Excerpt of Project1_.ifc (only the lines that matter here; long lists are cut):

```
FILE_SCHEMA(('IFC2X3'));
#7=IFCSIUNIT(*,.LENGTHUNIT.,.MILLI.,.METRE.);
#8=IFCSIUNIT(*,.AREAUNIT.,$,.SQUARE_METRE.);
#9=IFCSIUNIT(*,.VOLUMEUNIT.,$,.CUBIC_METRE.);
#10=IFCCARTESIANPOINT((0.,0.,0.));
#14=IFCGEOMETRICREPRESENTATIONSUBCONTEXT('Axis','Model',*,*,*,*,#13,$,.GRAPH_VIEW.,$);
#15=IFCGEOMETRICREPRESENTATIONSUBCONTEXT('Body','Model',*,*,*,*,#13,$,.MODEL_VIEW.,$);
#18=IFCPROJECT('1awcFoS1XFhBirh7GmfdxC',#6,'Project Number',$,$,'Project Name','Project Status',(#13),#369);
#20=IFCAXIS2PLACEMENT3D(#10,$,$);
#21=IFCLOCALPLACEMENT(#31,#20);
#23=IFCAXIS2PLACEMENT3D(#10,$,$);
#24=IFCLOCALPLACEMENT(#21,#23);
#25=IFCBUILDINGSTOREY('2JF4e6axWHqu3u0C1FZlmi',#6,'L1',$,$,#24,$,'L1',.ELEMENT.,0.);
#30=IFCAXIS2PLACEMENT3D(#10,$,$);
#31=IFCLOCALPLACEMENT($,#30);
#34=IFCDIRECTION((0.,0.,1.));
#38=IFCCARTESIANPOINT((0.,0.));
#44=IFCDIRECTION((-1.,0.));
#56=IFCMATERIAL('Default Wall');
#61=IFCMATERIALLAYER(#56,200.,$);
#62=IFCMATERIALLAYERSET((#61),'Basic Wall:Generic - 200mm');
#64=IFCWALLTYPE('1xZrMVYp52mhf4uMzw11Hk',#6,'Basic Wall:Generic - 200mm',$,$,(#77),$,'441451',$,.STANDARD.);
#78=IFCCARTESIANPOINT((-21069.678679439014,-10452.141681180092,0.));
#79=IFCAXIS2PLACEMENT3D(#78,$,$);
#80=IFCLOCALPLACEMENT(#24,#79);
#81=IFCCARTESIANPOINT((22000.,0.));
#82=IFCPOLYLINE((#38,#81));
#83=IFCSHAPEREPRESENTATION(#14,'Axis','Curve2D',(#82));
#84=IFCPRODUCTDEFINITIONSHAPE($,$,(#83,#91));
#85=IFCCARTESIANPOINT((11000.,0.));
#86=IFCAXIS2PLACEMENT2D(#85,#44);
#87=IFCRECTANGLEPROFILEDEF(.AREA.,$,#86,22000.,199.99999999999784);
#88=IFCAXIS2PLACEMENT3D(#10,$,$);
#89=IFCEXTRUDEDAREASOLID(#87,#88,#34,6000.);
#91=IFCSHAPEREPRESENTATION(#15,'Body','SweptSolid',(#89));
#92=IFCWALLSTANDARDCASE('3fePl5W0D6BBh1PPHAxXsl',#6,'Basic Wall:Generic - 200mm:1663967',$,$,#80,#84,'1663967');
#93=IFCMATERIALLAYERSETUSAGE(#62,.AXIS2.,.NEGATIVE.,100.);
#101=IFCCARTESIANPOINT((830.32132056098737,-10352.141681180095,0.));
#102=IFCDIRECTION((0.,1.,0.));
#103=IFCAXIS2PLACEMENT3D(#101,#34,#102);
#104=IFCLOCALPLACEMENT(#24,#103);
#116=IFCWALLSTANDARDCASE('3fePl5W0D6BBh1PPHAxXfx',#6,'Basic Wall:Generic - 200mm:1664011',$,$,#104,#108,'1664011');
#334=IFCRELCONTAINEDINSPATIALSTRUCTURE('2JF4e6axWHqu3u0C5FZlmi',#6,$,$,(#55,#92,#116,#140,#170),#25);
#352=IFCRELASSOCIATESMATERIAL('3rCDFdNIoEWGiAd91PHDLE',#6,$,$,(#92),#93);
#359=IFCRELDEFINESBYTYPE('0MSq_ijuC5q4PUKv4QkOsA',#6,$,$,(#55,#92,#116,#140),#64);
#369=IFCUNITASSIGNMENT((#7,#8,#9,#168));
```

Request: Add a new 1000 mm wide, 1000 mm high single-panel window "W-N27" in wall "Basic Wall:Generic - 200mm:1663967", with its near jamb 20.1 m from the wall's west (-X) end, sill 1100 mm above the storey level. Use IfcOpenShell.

```python
import numpy as np
import ifcopenshell
import ifcopenshell.api.feature
import ifcopenshell.api.geometry
import ifcopenshell.api.root
import ifcopenshell.api.spatial
import ifcopenshell.api.type
import ifcopenshell.geom
import ifcopenshell.util.element
import ifcopenshell.util.placement
import ifcopenshell.util.representation
import ifcopenshell.util.shape
import ifcopenshell.util.unit

model = ifcopenshell.open("Project1_.ifc")
unit_scale = ifcopenshell.util.unit.calculate_unit_scale(model)
settings = ifcopenshell.geom.settings()


def volume(element):
    """Net volume in cubic metres, openings subtracted."""
    shape = ifcopenshell.geom.create_shape(settings, element)
    return ifcopenshell.util.shape.get_volume(shape.geometry)


wall = model.by_guid("3fePl5W0D6BBh1PPHAxXsl")
storey = ifcopenshell.util.element.get_container(wall, ifc_class="IfcBuildingStorey")
context = ifcopenshell.util.representation.get_context(model, "Model", "Body", "MODEL_VIEW")
before = volume(wall)

width, height, from_end, sill = 1, 1, 20.1, 1.1  # metres

# The wall runs along its own X axis, and the end named is its -X end.
wall_shape = ifcopenshell.geom.create_shape(settings, wall)
x, y, z = ifcopenshell.util.shape.get_vertices(wall_shape.geometry).T
start = x.min() + from_end
face, thickness = float(y.min()), float(y.max() - y.min())
wall_matrix = ifcopenshell.util.placement.get_local_placement(wall.ObjectPlacement)
level = ifcopenshell.util.placement.get_local_placement(storey.ObjectPlacement)[2, 3]


def in_wall(x, y):
    """Placement at x, y metres in the wall's axes, at sill height."""
    matrix = wall_matrix.copy()
    matrix[:, 3] = wall_matrix @ np.array([x / unit_scale, y / unit_scale, 0.0, 1.0])
    matrix[2, 3] = level + sill / unit_scale
    return matrix


# Opening: a box that overshoots both wall faces by 50 mm.
opening = ifcopenshell.api.root.create_entity(model, ifc_class="IfcOpeningElement")
box = ifcopenshell.api.geometry.add_wall_representation(
    model, context=context, length=width, height=height, thickness=thickness + 0.1
)
ifcopenshell.api.geometry.assign_representation(model, product=opening, representation=box)
ifcopenshell.api.geometry.edit_object_placement(model, product=opening, matrix=in_wall(start, face - 0.05), is_si=False)
ifcopenshell.api.feature.add_feature(model, feature=opening, element=wall)

window = ifcopenshell.api.root.create_entity(model, ifc_class="IfcWindow", name="W-N27")
window.OverallWidth, window.OverallHeight = width / unit_scale, height / unit_scale
body = ifcopenshell.api.geometry.add_window_representation(
    model,
    context=context,
    overall_width=window.OverallWidth,
    overall_height=window.OverallHeight,
    partition_type="SINGLE_PANEL",
)
ifcopenshell.api.geometry.assign_representation(model, product=window, representation=body)
ifcopenshell.api.spatial.assign_container(model, products=[window], relating_structure=storey)
fills = ifcopenshell.api.feature.add_filling(model, opening=opening, element=window)
fills.OwnerHistory = window.OwnerHistory  # required in IFC2X3

# IFC2X3 keeps the operation on the window style.
style = ifcopenshell.api.root.create_entity(model, ifc_class="IfcWindowStyle", name="W-N27")
style.OperationType, style.ConstructionType = "SINGLE_PANEL", "NOTDEFINED"
style.ParameterTakesPrecedence = style.Sizeable = False
ifcopenshell.api.type.assign_type(model, related_objects=[window], relating_type=style)

# Centre the window in the wall's thickness.
ifcopenshell.api.geometry.edit_object_placement(model, product=window, matrix=in_wall(start, face), is_si=False)
window_shape = ifcopenshell.geom.create_shape(settings, window)
depth = ifcopenshell.util.shape.get_vertices(window_shape.geometry)[:, 1]
offset = face + thickness / 2 - (depth.min() + depth.max()) / 2
ifcopenshell.api.geometry.edit_object_placement(model, product=window, matrix=in_wall(start, offset), is_si=False)

after = volume(wall)

print(f"wall volume {before:.3f} -> {after:.3f} m3")

model.write("Project1__v2.ifc")
```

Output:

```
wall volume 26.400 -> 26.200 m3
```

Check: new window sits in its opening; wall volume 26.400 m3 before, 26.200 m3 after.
